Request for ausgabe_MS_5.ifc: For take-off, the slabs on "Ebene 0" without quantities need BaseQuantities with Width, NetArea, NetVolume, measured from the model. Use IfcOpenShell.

First a look at what the model holds.

```python
import ifcopenshell
import ifcopenshell.util.element
import ifcopenshell.util.unit

model = ifcopenshell.open("ausgabe_MS_5.ifc")
print(model.schema)
for unit_type in ("LENGTHUNIT", "AREAUNIT", "VOLUMEUNIT"):
    print(unit_type, ifcopenshell.util.unit.calculate_unit_scale(model, unit_type))
storey = next(s for s in model.by_type("IfcBuildingStorey") if s.Name == "Ebene 0")
slabs = [e for e in ifcopenshell.util.element.get_decomposition(storey) if e.is_a("IfcSlab")]
for e in sorted(slabs, key=lambda e: e.id()):
    print(e.id(), e.is_a(), e.Name, list(ifcopenshell.util.element.get_psets(e, qtos_only=True)), sep=" | ")
```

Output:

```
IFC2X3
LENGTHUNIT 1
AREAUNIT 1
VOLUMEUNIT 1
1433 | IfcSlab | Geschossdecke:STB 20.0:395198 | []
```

```python
import ifcopenshell
import ifcopenshell.api.pset
import ifcopenshell.geom
import ifcopenshell.util.element
import ifcopenshell.util.shape
import ifcopenshell.util.unit

model = ifcopenshell.open("ausgabe_MS_5.ifc")
unit_scale = ifcopenshell.util.unit.calculate_unit_scale(model)
area_scale = ifcopenshell.util.unit.calculate_unit_scale(model, "AREAUNIT")
volume_scale = ifcopenshell.util.unit.calculate_unit_scale(model, "VOLUMEUNIT")
settings = ifcopenshell.geom.settings()

storey = next(s for s in model.by_type("IfcBuildingStorey") if s.Name == "Ebene 0")
slabs = [e for e in ifcopenshell.util.element.get_decomposition(storey) if e.is_a("IfcSlab")]

for e in sorted(slabs, key=lambda e: e.id()):
    if ifcopenshell.util.element.get_psets(e, qtos_only=True, should_inherit=False):
        continue
    # Geometry comes back in metres, in the element's own axes.
    shape = ifcopenshell.geom.create_shape(settings, e)
    values = {
        "Width": ifcopenshell.util.shape.get_z(shape.geometry) / unit_scale,
        "NetArea": ifcopenshell.util.shape.get_footprint_area(shape.geometry) / area_scale,
        "NetVolume": ifcopenshell.util.shape.get_volume(shape.geometry) / volume_scale,
    }
    qto = ifcopenshell.api.pset.add_qto(model, product=e, name="BaseQuantities")
    ifcopenshell.api.pset.edit_qto(model, qto=qto, properties=values)
    print(e.id(), {k: round(v, 3) for k, v in values.items()})

model.write("ausgabe_MS_5_rev.ifc")
```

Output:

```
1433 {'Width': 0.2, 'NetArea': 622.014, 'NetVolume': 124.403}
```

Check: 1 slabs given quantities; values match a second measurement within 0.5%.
